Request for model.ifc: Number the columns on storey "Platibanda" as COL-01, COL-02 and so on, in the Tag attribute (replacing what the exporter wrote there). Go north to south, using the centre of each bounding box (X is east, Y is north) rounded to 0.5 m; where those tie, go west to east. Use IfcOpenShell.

First a look at what the model holds.

```python
import ifcopenshell
import ifcopenshell.util.element
import ifcopenshell.util.placement

model = ifcopenshell.open("model.ifc")
print(model.schema)
storey = next(s for s in model.by_type("IfcBuildingStorey") if s.Name == "Platibanda")
columns = [e for e in ifcopenshell.util.element.get_decomposition(storey) if e.is_a("IfcColumn")]
for e in sorted(columns, key=lambda e: e.id()):
    origin = ifcopenshell.util.placement.get_local_placement(e.ObjectPlacement)[:3, 3]
    print(e.id(), e.Tag, e.Name, origin.round(2) + 0.0, sep=" | ")
```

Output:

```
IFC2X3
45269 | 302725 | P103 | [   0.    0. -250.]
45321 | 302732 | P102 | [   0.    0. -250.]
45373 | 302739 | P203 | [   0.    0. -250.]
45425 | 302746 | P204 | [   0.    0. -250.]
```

```python
import ifcopenshell
import ifcopenshell.geom
import ifcopenshell.util.element
import ifcopenshell.util.shape

model = ifcopenshell.open("model.ifc")
settings = ifcopenshell.geom.settings()
settings.set("use-world-coords", True)


def centre(element):
    shape = ifcopenshell.geom.create_shape(settings, element)
    return ifcopenshell.util.shape.get_bbox_centroid(shape.geometry)


storey = next(s for s in model.by_type("IfcBuildingStorey") if s.Name == "Platibanda")
columns = [e for e in ifcopenshell.util.element.get_decomposition(storey) if e.is_a("IfcColumn")]

# Insertion points can sit at a corner or the storey origin, so sort by the geometry (in metres).
centres = {e: centre(e) for e in columns}
columns.sort(key=lambda e: (-round(centres[e][1] / 0.5), centres[e][0]))

for i, e in enumerate(columns, start=1):
    number = f"COL-{i:02d}"
    e.Tag = number
    print(e.id(), number)

model.write("model_rev.ifc")
```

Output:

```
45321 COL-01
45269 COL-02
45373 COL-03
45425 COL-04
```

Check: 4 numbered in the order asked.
